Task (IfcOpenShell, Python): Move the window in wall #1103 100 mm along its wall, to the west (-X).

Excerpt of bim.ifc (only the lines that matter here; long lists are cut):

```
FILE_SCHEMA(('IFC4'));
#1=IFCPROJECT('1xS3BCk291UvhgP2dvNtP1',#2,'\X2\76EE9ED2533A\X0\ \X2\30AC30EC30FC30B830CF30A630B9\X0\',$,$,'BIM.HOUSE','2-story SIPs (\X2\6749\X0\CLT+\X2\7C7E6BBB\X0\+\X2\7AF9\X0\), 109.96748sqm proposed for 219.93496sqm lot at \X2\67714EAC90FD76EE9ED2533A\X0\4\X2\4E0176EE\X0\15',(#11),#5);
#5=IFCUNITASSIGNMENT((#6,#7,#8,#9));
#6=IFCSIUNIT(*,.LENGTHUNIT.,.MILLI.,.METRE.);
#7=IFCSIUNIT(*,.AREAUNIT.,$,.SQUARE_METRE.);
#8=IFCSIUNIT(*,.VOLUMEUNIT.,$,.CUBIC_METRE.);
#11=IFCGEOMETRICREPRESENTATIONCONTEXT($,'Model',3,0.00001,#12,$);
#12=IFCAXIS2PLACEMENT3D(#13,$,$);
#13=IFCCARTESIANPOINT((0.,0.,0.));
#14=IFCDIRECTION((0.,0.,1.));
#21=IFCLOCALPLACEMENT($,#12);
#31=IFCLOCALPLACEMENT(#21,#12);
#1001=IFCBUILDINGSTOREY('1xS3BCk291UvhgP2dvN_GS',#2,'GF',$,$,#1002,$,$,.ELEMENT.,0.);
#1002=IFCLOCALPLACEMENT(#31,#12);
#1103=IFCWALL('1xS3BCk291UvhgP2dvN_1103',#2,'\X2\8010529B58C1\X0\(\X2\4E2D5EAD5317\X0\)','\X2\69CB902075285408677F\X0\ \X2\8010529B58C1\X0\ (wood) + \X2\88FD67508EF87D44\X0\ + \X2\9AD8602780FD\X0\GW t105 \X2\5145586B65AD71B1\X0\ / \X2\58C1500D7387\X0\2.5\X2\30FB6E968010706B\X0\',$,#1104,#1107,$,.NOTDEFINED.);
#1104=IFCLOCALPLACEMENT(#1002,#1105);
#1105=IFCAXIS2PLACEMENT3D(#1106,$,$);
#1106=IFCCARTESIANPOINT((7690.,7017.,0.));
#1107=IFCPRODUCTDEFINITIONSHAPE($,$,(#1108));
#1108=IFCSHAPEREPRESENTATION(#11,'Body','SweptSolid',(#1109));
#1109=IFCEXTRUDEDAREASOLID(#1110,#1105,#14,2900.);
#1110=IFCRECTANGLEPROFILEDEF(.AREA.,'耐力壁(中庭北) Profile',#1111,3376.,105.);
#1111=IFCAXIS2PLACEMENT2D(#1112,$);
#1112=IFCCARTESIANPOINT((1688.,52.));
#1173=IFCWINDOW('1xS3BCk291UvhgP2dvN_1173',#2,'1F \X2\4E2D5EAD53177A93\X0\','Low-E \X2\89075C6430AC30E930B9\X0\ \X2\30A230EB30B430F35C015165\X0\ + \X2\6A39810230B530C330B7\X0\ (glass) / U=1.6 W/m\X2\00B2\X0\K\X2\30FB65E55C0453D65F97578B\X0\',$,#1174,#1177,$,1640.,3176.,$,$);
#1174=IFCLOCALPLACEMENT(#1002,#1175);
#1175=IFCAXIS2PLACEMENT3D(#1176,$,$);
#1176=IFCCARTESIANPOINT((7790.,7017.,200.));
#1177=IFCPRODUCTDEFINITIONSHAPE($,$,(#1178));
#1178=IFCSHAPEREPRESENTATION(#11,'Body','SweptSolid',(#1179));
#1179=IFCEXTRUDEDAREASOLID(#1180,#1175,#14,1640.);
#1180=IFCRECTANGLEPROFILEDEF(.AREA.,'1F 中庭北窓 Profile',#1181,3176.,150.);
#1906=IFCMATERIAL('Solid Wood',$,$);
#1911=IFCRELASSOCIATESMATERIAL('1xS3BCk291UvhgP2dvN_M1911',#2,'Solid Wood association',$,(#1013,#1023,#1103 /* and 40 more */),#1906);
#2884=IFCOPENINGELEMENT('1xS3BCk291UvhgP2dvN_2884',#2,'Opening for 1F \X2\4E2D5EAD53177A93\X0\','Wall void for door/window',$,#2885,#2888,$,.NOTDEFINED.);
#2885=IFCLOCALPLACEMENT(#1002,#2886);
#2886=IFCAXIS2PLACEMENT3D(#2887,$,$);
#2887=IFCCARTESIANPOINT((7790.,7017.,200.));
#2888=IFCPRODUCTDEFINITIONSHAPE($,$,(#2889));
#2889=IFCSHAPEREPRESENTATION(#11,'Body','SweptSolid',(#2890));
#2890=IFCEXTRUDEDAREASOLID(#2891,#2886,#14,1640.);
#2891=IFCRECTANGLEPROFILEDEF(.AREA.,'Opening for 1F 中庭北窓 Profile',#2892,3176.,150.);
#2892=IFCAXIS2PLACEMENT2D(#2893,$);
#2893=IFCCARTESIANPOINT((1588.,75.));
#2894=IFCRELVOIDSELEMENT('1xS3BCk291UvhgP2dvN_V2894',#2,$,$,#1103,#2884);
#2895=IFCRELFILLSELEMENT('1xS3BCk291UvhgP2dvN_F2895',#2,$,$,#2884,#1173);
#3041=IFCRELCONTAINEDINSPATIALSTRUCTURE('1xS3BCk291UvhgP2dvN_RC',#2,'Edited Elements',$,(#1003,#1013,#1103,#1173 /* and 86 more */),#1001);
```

```python
import ifcopenshell
import ifcopenshell.api.geometry
import ifcopenshell.util.placement
import ifcopenshell.util.unit

model = ifcopenshell.open("bim.ifc")
unit_scale = ifcopenshell.util.unit.calculate_unit_scale(model)

window = model.by_guid("1xS3BCk291UvhgP2dvN_1173")
opening = window.FillsVoids[0].RelatingOpeningElement
wall = opening.VoidsElements[0].RelatingBuildingElement

wall_matrix = ifcopenshell.util.placement.get_local_placement(wall.ObjectPlacement)
shift = wall_matrix[:3, 0] * -0.1 / unit_scale
before = ifcopenshell.util.placement.get_local_placement(window.ObjectPlacement)[:3, 3].copy()

# The window is not placed relative to its opening, so move both.
for product in (opening, window):
    matrix = ifcopenshell.util.placement.get_local_placement(product.ObjectPlacement)
    matrix[:3, 3] += shift
    ifcopenshell.api.geometry.edit_object_placement(model, product=product, matrix=matrix, is_si=False)

after = ifcopenshell.util.placement.get_local_placement(window.ObjectPlacement)[:3, 3]
print("window moved by", (after - before).round(3) + 0.0)

model.write("bim_edited.ifc")
```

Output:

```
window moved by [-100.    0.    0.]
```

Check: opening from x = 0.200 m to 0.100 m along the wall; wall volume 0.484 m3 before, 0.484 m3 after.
